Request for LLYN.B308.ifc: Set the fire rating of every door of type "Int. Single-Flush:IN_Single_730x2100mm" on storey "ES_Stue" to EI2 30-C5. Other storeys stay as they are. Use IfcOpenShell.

First a look at what the model holds.

```python
import ifcopenshell
import ifcopenshell.util.element

model = ifcopenshell.open("LLYN.B308.ifc")
print(model.schema)
storey = next(s for s in model.by_type("IfcBuildingStorey") if s.Name == "ES_Stue")
doors = [e for e in ifcopenshell.util.element.get_decomposition(storey) if e.is_a("IfcDoor")]
seen = {}
for e in doors:
    element_type = ifcopenshell.util.element.get_type(e)
    key = (element_type.Name if element_type != e and element_type else None, ifcopenshell.util.element.get_pset(e, "Pset_DoorCommon", "FireRating"))
    seen[key] = seen.get(key, 0) + 1
for (name, value), count in sorted(seen.items(), key=str):
    print(count, "x", name, "|", value)
```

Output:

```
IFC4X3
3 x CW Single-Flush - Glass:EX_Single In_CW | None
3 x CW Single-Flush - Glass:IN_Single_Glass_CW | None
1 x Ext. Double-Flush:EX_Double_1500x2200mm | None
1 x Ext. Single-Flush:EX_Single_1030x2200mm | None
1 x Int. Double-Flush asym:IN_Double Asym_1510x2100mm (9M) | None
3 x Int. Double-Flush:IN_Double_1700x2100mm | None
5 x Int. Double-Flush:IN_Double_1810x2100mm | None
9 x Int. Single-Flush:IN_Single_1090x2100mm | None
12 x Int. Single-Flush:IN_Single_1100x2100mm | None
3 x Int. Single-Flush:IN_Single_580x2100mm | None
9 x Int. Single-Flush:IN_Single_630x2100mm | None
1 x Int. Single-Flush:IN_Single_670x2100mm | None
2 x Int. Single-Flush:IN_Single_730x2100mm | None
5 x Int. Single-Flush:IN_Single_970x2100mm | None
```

```python
import ifcopenshell
import ifcopenshell.api.pset
import ifcopenshell.util.element

model = ifcopenshell.open("LLYN.B308.ifc")

storey = next(s for s in model.by_type("IfcBuildingStorey") if s.Name == "ES_Stue")
doors = [e for e in ifcopenshell.util.element.get_decomposition(storey) if e.is_a("IfcDoor")]

count = 0
for e in doors:
    element_type = ifcopenshell.util.element.get_type(e)
    if element_type in (None, e) or element_type.Name != "Int. Single-Flush:IN_Single_730x2100mm":
        continue
    # add_pset returns the element's existing set when there is one.
    pset = ifcopenshell.api.pset.add_pset(model, product=e, name="Pset_DoorCommon")
    ifcopenshell.api.pset.edit_pset(model, pset=pset, properties={"FireRating": "EI2 30-C5"})
    count += 1

print(count, "doors updated")

model.write("LLYN.B308-out.ifc")
```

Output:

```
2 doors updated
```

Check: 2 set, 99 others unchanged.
